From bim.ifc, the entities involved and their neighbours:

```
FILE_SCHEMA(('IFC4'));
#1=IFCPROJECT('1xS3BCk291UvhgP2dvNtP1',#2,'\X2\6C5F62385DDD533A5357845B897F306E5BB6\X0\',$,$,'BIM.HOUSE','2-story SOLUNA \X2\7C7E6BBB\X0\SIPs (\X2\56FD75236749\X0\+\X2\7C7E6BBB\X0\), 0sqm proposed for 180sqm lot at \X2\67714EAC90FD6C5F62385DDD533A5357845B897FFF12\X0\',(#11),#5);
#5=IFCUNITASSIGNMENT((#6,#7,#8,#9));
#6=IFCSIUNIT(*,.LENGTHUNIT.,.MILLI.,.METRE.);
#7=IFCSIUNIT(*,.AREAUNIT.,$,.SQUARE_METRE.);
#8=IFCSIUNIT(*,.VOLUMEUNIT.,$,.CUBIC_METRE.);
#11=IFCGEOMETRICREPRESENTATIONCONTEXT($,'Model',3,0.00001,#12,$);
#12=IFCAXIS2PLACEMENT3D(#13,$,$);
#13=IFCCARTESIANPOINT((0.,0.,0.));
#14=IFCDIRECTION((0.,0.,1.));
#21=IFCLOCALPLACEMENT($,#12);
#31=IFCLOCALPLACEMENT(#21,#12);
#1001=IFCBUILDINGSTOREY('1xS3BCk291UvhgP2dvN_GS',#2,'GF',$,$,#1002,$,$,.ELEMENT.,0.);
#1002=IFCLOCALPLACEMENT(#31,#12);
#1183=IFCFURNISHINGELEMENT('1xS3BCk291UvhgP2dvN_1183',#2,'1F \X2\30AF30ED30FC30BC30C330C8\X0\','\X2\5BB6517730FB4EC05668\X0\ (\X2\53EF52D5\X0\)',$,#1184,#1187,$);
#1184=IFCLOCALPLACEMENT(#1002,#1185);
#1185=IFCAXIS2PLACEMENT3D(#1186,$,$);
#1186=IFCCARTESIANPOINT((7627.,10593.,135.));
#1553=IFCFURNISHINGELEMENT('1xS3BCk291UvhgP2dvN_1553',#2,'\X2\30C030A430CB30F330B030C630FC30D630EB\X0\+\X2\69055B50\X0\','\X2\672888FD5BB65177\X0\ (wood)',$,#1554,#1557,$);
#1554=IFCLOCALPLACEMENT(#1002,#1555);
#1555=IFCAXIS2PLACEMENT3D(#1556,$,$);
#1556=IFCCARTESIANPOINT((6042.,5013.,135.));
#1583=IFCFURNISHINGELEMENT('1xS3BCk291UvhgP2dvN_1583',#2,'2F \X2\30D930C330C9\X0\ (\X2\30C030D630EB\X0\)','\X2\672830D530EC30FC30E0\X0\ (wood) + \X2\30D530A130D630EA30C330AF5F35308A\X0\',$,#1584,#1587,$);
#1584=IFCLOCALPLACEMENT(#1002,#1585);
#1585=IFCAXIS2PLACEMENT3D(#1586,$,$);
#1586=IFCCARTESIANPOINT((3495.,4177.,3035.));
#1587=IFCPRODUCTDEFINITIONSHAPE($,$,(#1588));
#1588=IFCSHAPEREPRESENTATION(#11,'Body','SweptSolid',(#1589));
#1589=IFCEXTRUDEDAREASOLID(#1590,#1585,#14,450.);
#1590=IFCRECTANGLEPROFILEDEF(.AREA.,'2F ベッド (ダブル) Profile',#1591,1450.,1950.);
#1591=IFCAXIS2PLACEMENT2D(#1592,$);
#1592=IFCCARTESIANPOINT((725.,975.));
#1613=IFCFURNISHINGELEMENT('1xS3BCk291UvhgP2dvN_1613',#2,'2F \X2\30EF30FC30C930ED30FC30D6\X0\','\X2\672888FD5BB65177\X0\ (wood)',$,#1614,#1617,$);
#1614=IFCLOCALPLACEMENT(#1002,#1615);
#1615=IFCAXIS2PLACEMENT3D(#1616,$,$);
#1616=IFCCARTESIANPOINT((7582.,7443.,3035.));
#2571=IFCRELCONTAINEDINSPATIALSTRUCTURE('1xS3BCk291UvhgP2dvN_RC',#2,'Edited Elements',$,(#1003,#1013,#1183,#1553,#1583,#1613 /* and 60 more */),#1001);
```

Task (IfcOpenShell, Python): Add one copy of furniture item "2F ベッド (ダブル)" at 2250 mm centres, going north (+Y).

```python
import numpy as np
import ifcopenshell
import ifcopenshell.api.geometry
import ifcopenshell.api.root
import ifcopenshell.util.element
import ifcopenshell.util.placement
import ifcopenshell.util.unit

model = ifcopenshell.open("bim.ifc")
unit_scale = ifcopenshell.util.unit.calculate_unit_scale(model)


def reuse_history(source, copy):
    """copy_class also copies each property set's owner history, people and application; keep the originals."""
    for rel in copy.IsDefinedBy:
        if rel.is_a("IfcRelDefinesByProperties") and (history := rel.RelatingPropertyDefinition.OwnerHistory):
            rel.RelatingPropertyDefinition.OwnerHistory = source.OwnerHistory
            ifcopenshell.util.element.remove_deep2(model, history)


source = model.by_id(1583)
base = ifcopenshell.util.placement.get_local_placement(source.ObjectPlacement)
step = np.array([0.0, 1.0, 0.0]) * 2.25 / unit_scale

for i in range(1, 2):
    copy = ifcopenshell.api.root.copy_class(model, product=source)
    copy.Representation = ifcopenshell.util.element.copy_deep(
        model, source.Representation, exclude=["IfcGeometricRepresentationContext", "IfcRepresentationMap"]
    )
    reuse_history(source, copy)
    matrix = base.copy()
    matrix[:3, 3] += i * step
    print("added at", matrix[:3, 3].round(3) + 0.0)
    ifcopenshell.api.geometry.edit_object_placement(model, product=copy, matrix=matrix, is_si=False)

model.write("bim-out.ifc")
```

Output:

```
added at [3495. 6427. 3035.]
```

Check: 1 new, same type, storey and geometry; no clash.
